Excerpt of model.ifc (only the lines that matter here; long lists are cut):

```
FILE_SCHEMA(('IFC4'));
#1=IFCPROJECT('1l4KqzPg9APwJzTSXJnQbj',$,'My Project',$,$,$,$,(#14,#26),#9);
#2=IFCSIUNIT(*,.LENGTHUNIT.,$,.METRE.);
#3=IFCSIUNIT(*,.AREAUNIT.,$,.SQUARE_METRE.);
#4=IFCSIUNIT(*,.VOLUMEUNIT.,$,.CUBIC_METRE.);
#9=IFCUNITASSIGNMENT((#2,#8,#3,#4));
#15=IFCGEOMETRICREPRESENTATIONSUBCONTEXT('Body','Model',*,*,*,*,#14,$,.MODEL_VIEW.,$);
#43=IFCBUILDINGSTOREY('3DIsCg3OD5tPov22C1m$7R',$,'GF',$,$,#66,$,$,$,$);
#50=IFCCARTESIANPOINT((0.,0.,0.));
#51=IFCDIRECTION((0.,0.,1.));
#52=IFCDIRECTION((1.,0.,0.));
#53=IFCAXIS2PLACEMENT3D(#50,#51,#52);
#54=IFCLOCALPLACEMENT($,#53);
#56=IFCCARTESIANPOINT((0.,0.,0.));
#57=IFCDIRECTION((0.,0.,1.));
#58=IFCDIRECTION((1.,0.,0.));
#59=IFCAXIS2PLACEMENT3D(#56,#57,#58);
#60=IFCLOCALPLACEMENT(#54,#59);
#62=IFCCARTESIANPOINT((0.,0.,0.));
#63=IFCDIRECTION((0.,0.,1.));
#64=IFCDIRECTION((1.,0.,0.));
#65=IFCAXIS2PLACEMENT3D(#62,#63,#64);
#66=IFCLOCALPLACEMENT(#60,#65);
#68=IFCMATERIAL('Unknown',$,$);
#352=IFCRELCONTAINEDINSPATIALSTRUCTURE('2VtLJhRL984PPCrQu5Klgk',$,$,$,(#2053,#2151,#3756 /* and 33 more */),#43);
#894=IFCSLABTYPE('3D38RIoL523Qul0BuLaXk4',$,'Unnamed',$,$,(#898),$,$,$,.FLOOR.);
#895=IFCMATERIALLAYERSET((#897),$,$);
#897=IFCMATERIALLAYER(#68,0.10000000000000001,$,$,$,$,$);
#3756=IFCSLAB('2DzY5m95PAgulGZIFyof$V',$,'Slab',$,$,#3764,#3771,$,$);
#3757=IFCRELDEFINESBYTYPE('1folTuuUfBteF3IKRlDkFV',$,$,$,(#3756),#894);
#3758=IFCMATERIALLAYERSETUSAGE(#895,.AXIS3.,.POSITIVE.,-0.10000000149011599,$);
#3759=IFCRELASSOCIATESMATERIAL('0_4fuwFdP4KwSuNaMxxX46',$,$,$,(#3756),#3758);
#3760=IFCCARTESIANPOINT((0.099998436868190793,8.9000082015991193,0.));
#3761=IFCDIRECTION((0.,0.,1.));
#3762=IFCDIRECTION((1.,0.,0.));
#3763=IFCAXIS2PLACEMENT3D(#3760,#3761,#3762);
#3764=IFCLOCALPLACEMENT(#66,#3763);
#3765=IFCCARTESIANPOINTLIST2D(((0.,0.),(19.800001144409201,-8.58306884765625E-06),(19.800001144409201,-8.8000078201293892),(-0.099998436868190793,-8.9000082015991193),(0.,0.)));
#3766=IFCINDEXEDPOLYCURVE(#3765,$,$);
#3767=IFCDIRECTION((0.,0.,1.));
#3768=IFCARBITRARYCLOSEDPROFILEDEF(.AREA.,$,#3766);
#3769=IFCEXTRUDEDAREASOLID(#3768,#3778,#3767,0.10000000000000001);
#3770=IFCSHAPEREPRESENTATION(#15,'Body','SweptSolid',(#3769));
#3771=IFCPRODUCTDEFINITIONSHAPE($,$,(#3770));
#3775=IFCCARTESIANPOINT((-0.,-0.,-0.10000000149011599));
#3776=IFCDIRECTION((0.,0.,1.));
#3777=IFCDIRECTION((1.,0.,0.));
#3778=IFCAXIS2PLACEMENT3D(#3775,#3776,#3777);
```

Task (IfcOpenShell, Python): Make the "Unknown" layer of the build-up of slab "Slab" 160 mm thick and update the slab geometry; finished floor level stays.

```python
import ifcopenshell
import ifcopenshell.util.element
import ifcopenshell.util.representation

model = ifcopenshell.open("model.ifc")

layer_set = model.by_id(895)
layer = next(l for l in layer_set.MaterialLayers if l.Material and l.Material.Name == "Unknown")
change = 0.16 - layer.LayerThickness
layer.LayerThickness += change

# Geometry does not follow the layer set by itself.
slabs = [e for e in ifcopenshell.util.element.get_elements_by_material(model, layer_set) if e.is_a("IfcSlab")]
for slab in sorted(slabs, key=lambda e: e.id()):
    body = ifcopenshell.util.representation.get_representation(slab, "Model", "Body")
    solid = body.Items[0]
    old_depth = solid.Depth
    solid.Depth += change
    # Extruded upwards: lower the start of the extrusion so the top stays.
    x, y, z = solid.Position.Location.Coordinates
    solid.Position.Location = model.createIfcCartesianPoint((x, y, z - change))
    print(slab.id(), f"{old_depth:g} -> {solid.Depth:g}")

# The layers are counted up from the underside, which has moved.
for usage in {ifcopenshell.util.element.get_material(slab) for slab in slabs}:
    usage.OffsetFromReferenceLine -= change

model.write("model_rev.ifc")
```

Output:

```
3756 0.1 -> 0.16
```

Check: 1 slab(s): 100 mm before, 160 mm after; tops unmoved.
